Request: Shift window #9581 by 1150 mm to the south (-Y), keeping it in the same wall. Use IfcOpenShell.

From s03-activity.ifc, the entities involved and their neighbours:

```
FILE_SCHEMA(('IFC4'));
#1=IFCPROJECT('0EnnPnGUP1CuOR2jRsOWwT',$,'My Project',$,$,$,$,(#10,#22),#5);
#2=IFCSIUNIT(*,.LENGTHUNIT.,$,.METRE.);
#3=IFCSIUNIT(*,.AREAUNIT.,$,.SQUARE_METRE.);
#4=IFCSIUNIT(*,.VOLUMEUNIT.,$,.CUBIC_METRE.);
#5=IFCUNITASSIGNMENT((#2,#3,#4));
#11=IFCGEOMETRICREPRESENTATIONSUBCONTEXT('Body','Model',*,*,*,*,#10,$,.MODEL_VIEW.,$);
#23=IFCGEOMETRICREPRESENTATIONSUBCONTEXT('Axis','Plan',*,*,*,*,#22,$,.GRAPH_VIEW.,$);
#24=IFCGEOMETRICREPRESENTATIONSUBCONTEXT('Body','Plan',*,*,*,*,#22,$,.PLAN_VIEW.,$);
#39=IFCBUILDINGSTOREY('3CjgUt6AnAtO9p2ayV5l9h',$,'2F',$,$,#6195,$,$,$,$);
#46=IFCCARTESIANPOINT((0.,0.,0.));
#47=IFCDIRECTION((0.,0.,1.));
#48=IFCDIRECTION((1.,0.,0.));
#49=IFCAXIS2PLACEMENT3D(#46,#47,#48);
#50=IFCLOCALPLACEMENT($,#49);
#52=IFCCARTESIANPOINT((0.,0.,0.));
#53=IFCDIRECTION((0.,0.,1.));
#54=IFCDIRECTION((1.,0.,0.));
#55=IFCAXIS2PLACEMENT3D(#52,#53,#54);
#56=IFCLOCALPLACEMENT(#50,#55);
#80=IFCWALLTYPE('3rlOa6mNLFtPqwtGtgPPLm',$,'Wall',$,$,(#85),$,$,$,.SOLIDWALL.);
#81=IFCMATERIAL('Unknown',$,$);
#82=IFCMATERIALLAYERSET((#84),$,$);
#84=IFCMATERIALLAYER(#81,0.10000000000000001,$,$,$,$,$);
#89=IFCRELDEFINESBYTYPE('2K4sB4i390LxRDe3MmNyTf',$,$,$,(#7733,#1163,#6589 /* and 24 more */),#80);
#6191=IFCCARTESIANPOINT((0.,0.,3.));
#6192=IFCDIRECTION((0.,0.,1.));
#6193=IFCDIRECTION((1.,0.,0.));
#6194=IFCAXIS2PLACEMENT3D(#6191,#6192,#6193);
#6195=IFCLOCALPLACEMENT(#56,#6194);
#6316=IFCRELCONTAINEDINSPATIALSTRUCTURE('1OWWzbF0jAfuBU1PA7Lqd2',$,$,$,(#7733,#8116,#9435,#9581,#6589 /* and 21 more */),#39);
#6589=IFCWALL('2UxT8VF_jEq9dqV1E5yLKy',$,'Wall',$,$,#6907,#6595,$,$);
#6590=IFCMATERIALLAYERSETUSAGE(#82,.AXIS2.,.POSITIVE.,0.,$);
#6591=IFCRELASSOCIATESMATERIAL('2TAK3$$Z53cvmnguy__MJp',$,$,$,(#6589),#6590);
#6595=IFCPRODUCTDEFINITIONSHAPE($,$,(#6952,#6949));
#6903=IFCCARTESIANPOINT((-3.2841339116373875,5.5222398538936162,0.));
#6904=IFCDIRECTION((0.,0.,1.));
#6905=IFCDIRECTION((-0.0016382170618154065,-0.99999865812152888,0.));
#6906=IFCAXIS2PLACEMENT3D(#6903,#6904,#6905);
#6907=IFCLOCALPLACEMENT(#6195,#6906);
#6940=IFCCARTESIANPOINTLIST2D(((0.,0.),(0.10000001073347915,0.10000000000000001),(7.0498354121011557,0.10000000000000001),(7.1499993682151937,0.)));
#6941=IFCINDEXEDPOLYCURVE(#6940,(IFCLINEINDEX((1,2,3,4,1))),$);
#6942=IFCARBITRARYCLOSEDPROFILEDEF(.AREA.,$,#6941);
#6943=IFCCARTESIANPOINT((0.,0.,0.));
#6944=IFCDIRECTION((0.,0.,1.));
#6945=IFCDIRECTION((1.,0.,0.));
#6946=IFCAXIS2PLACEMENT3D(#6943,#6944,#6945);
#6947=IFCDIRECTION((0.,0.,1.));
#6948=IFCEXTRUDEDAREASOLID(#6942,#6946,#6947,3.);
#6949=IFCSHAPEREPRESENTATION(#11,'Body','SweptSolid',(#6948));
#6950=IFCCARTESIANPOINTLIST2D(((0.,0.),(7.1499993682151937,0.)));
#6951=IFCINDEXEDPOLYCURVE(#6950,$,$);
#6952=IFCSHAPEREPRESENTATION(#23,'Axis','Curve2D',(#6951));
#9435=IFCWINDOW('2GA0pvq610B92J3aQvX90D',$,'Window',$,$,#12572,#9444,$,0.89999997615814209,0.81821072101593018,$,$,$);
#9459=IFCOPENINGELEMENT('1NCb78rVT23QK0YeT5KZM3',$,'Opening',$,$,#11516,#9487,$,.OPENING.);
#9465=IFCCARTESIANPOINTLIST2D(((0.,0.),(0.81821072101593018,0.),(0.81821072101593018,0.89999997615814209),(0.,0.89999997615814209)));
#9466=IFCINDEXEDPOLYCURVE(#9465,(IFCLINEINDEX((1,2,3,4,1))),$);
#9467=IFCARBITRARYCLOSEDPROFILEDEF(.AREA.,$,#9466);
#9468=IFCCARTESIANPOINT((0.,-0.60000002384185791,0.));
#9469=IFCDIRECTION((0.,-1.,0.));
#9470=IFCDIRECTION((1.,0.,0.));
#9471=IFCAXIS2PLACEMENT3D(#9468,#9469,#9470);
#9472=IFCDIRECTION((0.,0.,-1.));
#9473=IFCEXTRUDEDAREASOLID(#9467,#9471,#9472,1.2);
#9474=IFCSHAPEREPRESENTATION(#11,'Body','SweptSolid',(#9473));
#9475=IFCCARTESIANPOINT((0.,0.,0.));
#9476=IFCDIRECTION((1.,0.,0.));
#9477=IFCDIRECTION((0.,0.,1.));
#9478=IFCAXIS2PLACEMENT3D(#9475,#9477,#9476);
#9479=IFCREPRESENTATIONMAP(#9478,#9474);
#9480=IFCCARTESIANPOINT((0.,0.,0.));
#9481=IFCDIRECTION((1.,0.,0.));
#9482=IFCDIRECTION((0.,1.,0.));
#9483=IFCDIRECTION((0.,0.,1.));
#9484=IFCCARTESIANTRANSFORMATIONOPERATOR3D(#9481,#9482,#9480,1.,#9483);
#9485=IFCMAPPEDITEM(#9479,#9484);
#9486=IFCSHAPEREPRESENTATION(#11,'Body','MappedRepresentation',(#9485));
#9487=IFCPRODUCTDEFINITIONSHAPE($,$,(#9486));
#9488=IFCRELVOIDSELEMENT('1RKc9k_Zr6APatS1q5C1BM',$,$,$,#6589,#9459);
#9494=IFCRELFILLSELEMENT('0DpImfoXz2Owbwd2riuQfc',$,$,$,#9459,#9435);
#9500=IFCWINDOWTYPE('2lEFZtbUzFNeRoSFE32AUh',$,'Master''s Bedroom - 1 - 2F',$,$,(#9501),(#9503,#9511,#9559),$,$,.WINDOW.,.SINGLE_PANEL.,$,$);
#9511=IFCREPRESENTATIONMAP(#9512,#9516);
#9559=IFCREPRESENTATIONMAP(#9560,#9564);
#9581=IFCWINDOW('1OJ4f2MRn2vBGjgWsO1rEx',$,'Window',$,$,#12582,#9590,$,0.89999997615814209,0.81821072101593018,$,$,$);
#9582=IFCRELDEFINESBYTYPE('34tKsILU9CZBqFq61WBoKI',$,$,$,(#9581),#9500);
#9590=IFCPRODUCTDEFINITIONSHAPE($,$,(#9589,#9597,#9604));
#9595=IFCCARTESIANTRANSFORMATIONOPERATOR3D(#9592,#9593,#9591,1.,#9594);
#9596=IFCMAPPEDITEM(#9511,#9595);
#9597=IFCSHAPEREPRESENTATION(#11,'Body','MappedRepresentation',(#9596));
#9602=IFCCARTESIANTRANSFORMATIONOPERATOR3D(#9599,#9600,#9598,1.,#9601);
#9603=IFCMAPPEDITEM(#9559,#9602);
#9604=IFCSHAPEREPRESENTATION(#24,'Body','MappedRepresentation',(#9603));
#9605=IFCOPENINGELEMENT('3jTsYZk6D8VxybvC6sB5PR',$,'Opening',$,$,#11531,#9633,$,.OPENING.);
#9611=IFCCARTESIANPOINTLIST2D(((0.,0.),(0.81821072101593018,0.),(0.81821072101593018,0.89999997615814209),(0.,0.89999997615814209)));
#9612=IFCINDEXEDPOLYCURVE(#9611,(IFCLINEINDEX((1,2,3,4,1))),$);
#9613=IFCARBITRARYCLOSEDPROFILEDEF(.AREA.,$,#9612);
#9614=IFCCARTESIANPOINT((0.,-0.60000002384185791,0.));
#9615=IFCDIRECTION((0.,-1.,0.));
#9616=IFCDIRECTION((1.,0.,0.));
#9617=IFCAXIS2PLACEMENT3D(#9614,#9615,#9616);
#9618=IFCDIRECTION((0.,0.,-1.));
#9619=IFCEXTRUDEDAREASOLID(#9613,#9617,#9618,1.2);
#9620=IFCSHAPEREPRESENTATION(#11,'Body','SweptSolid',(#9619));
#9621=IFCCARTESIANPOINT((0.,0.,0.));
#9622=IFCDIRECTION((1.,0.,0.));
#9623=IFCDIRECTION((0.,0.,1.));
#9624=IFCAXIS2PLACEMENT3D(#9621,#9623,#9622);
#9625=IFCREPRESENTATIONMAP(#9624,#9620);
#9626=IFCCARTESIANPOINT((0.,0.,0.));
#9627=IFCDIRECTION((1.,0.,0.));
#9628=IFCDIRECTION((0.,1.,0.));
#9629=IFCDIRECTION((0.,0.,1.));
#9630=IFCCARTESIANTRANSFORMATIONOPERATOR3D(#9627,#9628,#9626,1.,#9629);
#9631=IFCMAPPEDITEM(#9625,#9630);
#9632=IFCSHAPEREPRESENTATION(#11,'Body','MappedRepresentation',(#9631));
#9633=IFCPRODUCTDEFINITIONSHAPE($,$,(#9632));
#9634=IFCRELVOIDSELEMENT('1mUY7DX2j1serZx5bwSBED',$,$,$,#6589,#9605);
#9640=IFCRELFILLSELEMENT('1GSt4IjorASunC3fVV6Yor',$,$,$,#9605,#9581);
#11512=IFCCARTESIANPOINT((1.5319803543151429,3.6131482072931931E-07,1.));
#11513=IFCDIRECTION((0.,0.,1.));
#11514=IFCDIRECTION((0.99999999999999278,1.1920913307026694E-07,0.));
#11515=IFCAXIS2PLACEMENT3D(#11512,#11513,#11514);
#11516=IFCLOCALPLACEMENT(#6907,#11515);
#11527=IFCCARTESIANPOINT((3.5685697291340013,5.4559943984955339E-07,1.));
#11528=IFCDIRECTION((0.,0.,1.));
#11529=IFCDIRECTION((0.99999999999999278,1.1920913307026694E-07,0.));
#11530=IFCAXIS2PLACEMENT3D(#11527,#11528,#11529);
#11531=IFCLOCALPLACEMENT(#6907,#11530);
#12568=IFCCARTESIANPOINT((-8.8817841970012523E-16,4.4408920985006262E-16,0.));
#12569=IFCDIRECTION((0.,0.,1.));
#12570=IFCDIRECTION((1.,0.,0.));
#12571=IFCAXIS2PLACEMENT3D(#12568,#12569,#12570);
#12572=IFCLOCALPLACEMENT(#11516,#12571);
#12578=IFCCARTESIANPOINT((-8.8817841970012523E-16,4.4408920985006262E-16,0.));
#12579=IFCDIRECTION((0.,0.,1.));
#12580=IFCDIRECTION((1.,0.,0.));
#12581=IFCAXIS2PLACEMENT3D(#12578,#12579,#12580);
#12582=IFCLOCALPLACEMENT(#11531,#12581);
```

```python
import ifcopenshell
import ifcopenshell.api.geometry
import ifcopenshell.util.placement

model = ifcopenshell.open("s03-activity.ifc")

window = model.by_guid("1OJ4f2MRn2vBGjgWsO1rEx")
opening = window.FillsVoids[0].RelatingOpeningElement
wall = opening.VoidsElements[0].RelatingBuildingElement

wall_matrix = ifcopenshell.util.placement.get_local_placement(wall.ObjectPlacement)
shift = wall_matrix[:3, 0] * 1.15
before = ifcopenshell.util.placement.get_local_placement(window.ObjectPlacement)[:3, 3].copy()

# The window is placed relative to its opening, so it follows when the opening moves.
matrix = ifcopenshell.util.placement.get_local_placement(opening.ObjectPlacement)
matrix[:3, 3] += shift
ifcopenshell.api.geometry.edit_object_placement(
    model, product=opening, matrix=matrix, is_si=False, should_transform_children=True
)

after = ifcopenshell.util.placement.get_local_placement(window.ObjectPlacement)[:3, 3]
print("window moved by", (after - before).round(3) + 0.0)

model.write("s03-activity_edited.ifc")
```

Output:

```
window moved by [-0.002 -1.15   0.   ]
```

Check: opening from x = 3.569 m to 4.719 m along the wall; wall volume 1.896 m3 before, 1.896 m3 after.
